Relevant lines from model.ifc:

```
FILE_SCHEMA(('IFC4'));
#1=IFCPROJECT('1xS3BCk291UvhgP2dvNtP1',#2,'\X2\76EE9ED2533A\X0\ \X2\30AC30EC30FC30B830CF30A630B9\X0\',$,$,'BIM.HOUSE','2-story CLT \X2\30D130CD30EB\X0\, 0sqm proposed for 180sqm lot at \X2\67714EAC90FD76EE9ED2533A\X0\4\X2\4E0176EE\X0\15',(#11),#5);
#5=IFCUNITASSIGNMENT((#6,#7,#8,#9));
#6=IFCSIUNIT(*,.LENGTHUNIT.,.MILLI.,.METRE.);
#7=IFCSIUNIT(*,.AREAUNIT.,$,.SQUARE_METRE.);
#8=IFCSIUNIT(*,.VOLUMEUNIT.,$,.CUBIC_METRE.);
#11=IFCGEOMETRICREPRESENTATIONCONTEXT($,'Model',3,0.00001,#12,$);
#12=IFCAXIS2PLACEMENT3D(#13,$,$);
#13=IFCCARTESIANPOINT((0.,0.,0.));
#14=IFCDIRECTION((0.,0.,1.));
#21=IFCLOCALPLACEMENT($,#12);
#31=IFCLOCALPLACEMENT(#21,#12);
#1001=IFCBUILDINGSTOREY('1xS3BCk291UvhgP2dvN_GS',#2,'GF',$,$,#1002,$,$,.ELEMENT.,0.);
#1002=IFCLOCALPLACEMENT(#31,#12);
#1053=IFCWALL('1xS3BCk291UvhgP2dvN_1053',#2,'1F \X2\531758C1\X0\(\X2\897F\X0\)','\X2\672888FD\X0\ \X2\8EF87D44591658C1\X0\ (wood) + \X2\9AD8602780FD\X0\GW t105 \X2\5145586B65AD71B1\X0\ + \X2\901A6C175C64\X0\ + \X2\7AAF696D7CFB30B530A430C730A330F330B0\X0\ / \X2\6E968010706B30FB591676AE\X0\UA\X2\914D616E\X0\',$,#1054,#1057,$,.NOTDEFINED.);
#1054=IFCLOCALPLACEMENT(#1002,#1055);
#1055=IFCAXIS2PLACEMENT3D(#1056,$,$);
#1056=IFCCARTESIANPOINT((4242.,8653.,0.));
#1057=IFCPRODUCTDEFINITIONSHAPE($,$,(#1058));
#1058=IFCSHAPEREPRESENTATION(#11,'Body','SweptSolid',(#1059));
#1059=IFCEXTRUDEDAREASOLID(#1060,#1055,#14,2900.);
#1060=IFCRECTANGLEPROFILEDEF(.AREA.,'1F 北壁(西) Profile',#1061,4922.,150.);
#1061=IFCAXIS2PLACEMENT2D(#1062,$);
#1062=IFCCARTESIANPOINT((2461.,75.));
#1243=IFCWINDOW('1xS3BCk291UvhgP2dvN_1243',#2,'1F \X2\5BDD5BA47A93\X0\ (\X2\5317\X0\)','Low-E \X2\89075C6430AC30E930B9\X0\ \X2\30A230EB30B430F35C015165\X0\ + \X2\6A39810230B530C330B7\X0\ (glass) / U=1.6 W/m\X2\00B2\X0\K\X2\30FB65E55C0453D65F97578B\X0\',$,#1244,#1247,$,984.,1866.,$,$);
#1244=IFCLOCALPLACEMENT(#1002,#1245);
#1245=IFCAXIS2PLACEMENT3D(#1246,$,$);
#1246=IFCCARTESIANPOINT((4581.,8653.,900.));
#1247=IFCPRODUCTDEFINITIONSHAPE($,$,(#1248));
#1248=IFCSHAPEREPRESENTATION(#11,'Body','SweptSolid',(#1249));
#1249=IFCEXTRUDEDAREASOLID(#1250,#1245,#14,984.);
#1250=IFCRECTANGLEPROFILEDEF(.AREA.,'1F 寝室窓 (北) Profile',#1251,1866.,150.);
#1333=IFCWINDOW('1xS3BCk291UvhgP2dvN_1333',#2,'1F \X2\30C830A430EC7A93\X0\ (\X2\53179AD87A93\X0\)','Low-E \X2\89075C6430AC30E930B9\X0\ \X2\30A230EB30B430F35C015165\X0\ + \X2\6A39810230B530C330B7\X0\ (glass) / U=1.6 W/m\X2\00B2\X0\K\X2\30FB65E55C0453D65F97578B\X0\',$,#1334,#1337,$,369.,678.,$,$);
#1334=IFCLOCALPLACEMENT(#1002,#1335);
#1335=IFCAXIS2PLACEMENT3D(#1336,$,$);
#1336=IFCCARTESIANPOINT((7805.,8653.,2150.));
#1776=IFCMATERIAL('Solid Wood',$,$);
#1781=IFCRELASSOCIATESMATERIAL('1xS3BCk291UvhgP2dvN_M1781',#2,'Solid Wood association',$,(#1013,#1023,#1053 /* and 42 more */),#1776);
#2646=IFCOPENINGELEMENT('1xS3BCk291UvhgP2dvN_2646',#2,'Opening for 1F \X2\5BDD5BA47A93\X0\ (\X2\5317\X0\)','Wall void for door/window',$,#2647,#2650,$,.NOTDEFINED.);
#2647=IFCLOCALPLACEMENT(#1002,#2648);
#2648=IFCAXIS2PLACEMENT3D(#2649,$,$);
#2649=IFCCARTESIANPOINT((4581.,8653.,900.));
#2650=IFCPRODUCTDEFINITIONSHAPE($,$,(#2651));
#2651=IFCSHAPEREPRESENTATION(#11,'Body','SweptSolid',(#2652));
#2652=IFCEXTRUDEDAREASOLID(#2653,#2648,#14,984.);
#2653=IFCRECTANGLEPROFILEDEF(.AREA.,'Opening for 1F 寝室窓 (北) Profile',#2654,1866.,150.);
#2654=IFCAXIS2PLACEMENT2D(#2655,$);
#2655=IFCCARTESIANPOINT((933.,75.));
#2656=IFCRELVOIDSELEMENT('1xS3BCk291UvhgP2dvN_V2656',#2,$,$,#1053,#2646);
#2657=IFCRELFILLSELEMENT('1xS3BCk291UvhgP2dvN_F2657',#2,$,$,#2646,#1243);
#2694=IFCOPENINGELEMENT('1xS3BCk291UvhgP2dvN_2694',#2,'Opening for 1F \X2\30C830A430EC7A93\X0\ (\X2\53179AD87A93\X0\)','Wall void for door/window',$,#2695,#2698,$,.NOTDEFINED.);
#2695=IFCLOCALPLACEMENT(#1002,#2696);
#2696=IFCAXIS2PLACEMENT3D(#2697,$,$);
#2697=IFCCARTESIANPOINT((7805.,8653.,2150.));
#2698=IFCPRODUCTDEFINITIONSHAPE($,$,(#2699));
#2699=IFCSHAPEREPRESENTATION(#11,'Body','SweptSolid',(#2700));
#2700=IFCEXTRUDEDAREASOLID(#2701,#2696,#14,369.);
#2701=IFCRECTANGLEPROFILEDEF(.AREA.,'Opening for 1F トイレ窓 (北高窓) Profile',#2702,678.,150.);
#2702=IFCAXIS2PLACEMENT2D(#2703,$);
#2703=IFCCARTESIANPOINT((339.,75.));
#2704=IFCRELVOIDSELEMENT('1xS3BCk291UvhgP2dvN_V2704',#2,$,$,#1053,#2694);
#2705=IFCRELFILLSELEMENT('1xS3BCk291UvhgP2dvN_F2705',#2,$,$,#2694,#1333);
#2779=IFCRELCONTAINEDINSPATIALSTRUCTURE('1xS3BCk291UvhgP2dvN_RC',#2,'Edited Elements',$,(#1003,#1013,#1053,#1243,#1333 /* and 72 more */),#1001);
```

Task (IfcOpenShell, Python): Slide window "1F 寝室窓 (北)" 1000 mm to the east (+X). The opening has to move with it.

```python
import ifcopenshell
import ifcopenshell.api.geometry
import ifcopenshell.util.placement

model = ifcopenshell.open("model.ifc")

window = model.by_guid("1xS3BCk291UvhgP2dvN_1243")
opening = window.FillsVoids[0].RelatingOpeningElement
wall = opening.VoidsElements[0].RelatingBuildingElement

wall_matrix = ifcopenshell.util.placement.get_local_placement(wall.ObjectPlacement)
shift = wall_matrix[:3, 0] * 1000.0
before = ifcopenshell.util.placement.get_local_placement(window.ObjectPlacement)[:3, 3].copy()

# The window is not placed relative to its opening, so move both.
for product in (opening, window):
    matrix = ifcopenshell.util.placement.get_local_placement(product.ObjectPlacement)
    matrix[:3, 3] += shift
    ifcopenshell.api.geometry.edit_object_placement(model, product=product, matrix=matrix, is_si=False)

after = ifcopenshell.util.placement.get_local_placement(window.ObjectPlacement)[:3, 3]
print("window moved by", (after - before).round(3) + 0.0)

model.write("model_updated.ifc")
```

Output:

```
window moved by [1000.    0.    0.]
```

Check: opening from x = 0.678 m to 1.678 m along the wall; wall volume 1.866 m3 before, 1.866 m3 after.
